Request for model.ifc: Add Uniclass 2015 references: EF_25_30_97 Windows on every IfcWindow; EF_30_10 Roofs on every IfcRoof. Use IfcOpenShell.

First a look at what the model holds.

```python
import ifcopenshell

model = ifcopenshell.open("model.ifc")
print(model.schema)
print("classifications:", [c.Name for c in model.by_type("IfcClassification")])
for ifc_class in ("IfcDoor", "IfcRoof", "IfcStair", "IfcWall", "IfcWindow"):
    print(ifc_class, len(model.by_type(ifc_class)))
```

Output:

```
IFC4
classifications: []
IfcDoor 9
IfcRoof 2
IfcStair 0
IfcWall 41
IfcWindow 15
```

```python
import ifcopenshell
import ifcopenshell.api.classification

model = ifcopenshell.open("model.ifc")

system = ifcopenshell.api.classification.add_classification(model, classification="Uniclass 2015")

codes = {
    "IfcWindow": ("EF_25_30_97", "Windows"),
    "IfcRoof": ("EF_30_10", "Roofs"),
}
for ifc_class, (code, name) in codes.items():
    products = model.by_type(ifc_class)
    ifcopenshell.api.classification.add_reference(
        model, products=products, classification=system, identification=code, name=name
    )
    print(code, len(products))

model.write("model-out.ifc")
```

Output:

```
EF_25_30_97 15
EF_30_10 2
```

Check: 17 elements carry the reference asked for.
